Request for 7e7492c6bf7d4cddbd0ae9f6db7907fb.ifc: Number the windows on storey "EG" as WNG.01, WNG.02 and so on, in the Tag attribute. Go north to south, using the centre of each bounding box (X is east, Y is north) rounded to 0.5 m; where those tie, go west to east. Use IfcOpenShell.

First a look at what the model holds.

```python
import ifcopenshell
import ifcopenshell.util.element
import ifcopenshell.util.placement

model = ifcopenshell.open("7e7492c6bf7d4cddbd0ae9f6db7907fb.ifc")
print(model.schema)
storey = next(s for s in model.by_type("IfcBuildingStorey") if s.Name == "EG")
windows = [e for e in ifcopenshell.util.element.get_decomposition(storey) if e.is_a("IfcWindow")]
for e in sorted(windows, key=lambda e: e.id()):
    origin = ifcopenshell.util.placement.get_local_placement(e.ObjectPlacement)[:3, 3]
    print(e.id(), e.Tag, e.Name, origin.round(2) + 0.0, sep=" | ")
```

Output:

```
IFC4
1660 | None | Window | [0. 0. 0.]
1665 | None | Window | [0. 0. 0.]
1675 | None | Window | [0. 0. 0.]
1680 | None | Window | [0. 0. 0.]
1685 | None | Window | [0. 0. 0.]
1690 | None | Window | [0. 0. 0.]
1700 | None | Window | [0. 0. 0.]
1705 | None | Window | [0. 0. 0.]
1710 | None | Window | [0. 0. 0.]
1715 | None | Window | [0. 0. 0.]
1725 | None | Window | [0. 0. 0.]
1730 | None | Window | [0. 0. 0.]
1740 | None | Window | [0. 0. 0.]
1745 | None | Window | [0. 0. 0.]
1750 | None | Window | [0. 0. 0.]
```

```python
import ifcopenshell
import ifcopenshell.geom
import ifcopenshell.util.element
import ifcopenshell.util.shape

model = ifcopenshell.open("7e7492c6bf7d4cddbd0ae9f6db7907fb.ifc")
settings = ifcopenshell.geom.settings()
settings.set("use-world-coords", True)


def centre(element):
    shape = ifcopenshell.geom.create_shape(settings, element)
    return ifcopenshell.util.shape.get_bbox_centroid(shape.geometry)


storey = next(s for s in model.by_type("IfcBuildingStorey") if s.Name == "EG")
windows = [e for e in ifcopenshell.util.element.get_decomposition(storey) if e.is_a("IfcWindow")]

# Insertion points can sit at a corner or the storey origin, so sort by the geometry (in metres).
centres = {e: centre(e) for e in windows}
windows.sort(key=lambda e: (-round(centres[e][1] / 0.5), centres[e][0]))

for i, e in enumerate(windows, start=1):
    number = f"WNG.{i:02d}"
    e.Tag = number
    print(e.id(), number)

model.write("7e7492c6bf7d4cddbd0ae9f6db7907fb-out.ifc")
```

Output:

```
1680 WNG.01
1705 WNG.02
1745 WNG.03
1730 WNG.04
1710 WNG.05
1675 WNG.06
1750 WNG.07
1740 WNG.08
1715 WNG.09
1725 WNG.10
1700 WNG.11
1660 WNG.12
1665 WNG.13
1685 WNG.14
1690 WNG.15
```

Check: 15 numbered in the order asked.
